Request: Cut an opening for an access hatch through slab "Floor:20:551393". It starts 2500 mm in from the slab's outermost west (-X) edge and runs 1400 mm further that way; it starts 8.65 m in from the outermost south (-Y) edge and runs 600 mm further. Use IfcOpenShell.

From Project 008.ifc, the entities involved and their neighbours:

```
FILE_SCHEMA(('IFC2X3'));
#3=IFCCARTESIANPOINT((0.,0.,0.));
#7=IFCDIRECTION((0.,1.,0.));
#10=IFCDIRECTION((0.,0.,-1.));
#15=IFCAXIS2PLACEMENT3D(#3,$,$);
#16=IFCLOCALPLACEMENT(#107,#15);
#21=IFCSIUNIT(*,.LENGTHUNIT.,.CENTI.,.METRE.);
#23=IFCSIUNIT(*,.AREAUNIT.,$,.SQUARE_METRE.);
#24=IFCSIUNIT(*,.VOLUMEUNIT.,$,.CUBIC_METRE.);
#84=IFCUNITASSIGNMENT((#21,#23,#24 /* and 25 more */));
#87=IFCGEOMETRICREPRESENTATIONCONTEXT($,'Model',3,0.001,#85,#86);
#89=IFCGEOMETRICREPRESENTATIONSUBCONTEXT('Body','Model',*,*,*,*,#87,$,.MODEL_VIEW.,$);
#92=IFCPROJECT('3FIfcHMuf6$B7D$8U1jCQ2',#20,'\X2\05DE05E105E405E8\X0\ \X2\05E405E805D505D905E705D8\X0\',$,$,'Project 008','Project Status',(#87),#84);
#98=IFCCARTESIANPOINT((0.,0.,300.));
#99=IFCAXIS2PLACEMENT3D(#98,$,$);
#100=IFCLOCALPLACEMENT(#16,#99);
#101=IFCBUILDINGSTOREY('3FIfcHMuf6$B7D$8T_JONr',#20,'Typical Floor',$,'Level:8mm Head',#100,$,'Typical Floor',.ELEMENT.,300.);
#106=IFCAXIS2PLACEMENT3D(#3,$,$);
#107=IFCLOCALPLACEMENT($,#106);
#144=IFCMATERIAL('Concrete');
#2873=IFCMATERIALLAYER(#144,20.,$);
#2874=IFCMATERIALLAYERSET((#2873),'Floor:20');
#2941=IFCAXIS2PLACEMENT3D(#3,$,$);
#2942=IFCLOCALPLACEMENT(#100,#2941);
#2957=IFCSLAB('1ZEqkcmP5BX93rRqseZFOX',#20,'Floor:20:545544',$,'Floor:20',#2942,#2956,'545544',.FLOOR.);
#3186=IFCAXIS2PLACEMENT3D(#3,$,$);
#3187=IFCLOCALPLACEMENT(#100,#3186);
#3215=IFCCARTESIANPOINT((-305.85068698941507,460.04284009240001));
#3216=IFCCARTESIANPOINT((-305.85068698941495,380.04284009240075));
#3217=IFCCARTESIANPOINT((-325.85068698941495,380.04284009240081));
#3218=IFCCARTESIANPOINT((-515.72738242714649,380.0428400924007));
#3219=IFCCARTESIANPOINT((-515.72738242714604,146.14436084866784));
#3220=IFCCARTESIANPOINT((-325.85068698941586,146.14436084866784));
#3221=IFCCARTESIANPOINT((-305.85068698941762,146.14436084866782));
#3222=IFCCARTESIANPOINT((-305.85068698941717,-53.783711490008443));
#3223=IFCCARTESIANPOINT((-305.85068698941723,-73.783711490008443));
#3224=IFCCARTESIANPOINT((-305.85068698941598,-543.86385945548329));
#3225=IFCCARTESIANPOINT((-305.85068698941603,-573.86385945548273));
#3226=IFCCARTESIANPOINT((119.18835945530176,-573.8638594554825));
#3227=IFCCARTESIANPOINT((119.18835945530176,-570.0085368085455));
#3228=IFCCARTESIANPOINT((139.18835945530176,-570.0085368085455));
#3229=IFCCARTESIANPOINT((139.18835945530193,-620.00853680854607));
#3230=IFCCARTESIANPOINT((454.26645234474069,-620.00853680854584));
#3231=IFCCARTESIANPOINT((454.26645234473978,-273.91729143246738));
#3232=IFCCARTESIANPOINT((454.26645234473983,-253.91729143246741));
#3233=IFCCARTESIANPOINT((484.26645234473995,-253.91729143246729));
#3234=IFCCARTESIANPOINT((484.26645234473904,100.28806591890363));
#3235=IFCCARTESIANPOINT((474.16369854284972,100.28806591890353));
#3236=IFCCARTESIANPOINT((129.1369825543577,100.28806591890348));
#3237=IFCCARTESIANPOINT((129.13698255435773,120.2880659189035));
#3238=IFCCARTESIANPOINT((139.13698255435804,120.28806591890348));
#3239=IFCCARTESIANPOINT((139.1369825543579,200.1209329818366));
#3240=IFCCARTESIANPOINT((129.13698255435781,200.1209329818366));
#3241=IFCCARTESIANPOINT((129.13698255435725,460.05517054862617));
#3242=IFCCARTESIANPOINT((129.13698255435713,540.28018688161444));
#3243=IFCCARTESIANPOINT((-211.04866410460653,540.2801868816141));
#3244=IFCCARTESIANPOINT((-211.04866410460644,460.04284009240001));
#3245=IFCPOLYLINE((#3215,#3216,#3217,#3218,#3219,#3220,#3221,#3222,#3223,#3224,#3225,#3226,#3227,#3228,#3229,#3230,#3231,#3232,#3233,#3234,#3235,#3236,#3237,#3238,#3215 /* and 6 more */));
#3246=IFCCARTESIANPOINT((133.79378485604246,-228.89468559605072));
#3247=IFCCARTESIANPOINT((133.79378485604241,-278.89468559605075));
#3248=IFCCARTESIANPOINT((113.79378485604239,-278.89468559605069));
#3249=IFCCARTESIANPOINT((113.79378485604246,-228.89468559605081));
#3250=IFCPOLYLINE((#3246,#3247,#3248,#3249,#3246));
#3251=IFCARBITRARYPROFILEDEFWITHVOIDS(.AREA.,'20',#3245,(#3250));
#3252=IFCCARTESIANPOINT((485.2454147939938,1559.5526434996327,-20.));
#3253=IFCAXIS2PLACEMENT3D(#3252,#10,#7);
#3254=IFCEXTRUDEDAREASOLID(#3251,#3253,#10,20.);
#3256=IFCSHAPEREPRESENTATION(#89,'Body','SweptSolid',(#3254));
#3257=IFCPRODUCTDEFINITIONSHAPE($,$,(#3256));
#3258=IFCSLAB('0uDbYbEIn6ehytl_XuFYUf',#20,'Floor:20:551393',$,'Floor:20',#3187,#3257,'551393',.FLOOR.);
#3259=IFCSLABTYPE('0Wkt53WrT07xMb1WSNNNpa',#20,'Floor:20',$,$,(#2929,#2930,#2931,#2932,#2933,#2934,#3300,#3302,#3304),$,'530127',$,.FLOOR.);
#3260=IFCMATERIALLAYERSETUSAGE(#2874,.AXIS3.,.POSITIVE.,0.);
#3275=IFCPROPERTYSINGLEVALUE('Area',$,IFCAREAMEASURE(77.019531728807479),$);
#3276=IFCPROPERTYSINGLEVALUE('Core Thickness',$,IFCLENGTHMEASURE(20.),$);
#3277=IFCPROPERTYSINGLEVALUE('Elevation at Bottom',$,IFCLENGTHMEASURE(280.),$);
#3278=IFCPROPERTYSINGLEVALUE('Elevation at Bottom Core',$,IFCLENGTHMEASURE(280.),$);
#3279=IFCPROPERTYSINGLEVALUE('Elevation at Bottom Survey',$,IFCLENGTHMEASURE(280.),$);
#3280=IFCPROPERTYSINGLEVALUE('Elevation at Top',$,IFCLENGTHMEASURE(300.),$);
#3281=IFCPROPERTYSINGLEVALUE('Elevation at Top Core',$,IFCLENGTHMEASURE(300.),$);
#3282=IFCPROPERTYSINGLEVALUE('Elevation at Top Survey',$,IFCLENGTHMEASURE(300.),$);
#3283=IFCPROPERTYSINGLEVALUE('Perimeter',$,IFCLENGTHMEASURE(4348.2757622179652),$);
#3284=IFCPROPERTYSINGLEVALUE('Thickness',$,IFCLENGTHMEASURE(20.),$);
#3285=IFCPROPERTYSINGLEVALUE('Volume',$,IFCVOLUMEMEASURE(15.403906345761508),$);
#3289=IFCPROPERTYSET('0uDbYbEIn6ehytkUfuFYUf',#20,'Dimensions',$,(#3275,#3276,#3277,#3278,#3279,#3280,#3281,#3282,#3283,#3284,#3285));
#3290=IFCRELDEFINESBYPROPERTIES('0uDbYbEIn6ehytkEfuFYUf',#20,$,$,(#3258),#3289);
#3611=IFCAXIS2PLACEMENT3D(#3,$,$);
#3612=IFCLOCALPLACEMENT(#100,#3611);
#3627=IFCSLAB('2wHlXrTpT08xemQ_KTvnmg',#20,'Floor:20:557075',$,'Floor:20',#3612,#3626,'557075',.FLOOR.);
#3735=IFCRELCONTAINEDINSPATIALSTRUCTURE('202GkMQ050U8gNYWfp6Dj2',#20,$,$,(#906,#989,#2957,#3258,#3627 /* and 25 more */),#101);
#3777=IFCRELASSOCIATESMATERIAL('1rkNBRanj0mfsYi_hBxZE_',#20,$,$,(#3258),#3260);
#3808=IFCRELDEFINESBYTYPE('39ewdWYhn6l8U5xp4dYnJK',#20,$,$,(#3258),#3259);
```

```python
import numpy as np
import ifcopenshell
import ifcopenshell.api.feature
import ifcopenshell.api.geometry
import ifcopenshell.api.pset
import ifcopenshell.api.root
import ifcopenshell.geom
import ifcopenshell.util.element
import ifcopenshell.util.placement
import ifcopenshell.util.representation
import ifcopenshell.util.shape
import ifcopenshell.util.unit

model = ifcopenshell.open("Project 008.ifc")
unit_scale = ifcopenshell.util.unit.calculate_unit_scale(model)
area_scale = ifcopenshell.util.unit.calculate_unit_scale(model, "AREAUNIT")
volume_scale = ifcopenshell.util.unit.calculate_unit_scale(model, "VOLUMEUNIT")
settings = ifcopenshell.geom.settings()


def volume(element):
    """Net volume in cubic metres, openings subtracted."""
    shape = ifcopenshell.geom.create_shape(settings, element)
    return ifcopenshell.util.shape.get_volume(shape.geometry)


slab = model.by_guid("0uDbYbEIn6ehytl_XuFYUf")
before = volume(slab)

# Extent in the slab's own axes, in metres. The edges named are its -X and -Y sides.
slab_shape = ifcopenshell.geom.create_shape(settings, slab)
vertices = ifcopenshell.util.shape.get_vertices(slab_shape.geometry)
x_min, y_min, bottom = vertices.min(axis=0)
top = vertices[:, 2].max()

opening = ifcopenshell.api.root.create_entity(model, ifc_class="IfcOpeningElement", name="Access hatch opening")
context = ifcopenshell.util.representation.get_context(model, "Model", "Body", "MODEL_VIEW")
width, depth = 1.4, 0.6
outline = [(0.0, 0.0), (width, 0.0), (width, depth), (0.0, depth), (0.0, 0.0)]
# Overshoot both faces by 50 mm so the cut is clean.
shape = ifcopenshell.api.geometry.add_slab_representation(
    model, context=context, depth=top - bottom + 0.1, polyline=outline
)
ifcopenshell.api.geometry.assign_representation(model, product=opening, representation=shape)

matrix = ifcopenshell.util.placement.get_local_placement(slab.ObjectPlacement)
matrix[:, 3] = matrix @ np.append(np.array([x_min + 2.5, y_min + 8.65, bottom - 0.05]) / unit_scale, 1.0)
ifcopenshell.api.geometry.edit_object_placement(model, product=opening, matrix=matrix, is_si=False)
ifcopenshell.api.feature.add_feature(model, feature=opening, element=slab)

after = volume(slab)

# Update the slab's stored quantities.
pset = model.by_id(ifcopenshell.util.element.get_pset(slab, "Dimensions", should_inherit=False)["id"])
ifcopenshell.api.pset.edit_pset(model, pset=pset, properties={
    "Area": model.create_entity("IfcAreaMeasure", after / (top - bottom) / area_scale),
    "Volume": model.create_entity("IfcVolumeMeasure", after / volume_scale),
})

print(f"slab volume {before:.3f} -> {after:.3f} m3")

model.write("Project 008_updated.ifc")
```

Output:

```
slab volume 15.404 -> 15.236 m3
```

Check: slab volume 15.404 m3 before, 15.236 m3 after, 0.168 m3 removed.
